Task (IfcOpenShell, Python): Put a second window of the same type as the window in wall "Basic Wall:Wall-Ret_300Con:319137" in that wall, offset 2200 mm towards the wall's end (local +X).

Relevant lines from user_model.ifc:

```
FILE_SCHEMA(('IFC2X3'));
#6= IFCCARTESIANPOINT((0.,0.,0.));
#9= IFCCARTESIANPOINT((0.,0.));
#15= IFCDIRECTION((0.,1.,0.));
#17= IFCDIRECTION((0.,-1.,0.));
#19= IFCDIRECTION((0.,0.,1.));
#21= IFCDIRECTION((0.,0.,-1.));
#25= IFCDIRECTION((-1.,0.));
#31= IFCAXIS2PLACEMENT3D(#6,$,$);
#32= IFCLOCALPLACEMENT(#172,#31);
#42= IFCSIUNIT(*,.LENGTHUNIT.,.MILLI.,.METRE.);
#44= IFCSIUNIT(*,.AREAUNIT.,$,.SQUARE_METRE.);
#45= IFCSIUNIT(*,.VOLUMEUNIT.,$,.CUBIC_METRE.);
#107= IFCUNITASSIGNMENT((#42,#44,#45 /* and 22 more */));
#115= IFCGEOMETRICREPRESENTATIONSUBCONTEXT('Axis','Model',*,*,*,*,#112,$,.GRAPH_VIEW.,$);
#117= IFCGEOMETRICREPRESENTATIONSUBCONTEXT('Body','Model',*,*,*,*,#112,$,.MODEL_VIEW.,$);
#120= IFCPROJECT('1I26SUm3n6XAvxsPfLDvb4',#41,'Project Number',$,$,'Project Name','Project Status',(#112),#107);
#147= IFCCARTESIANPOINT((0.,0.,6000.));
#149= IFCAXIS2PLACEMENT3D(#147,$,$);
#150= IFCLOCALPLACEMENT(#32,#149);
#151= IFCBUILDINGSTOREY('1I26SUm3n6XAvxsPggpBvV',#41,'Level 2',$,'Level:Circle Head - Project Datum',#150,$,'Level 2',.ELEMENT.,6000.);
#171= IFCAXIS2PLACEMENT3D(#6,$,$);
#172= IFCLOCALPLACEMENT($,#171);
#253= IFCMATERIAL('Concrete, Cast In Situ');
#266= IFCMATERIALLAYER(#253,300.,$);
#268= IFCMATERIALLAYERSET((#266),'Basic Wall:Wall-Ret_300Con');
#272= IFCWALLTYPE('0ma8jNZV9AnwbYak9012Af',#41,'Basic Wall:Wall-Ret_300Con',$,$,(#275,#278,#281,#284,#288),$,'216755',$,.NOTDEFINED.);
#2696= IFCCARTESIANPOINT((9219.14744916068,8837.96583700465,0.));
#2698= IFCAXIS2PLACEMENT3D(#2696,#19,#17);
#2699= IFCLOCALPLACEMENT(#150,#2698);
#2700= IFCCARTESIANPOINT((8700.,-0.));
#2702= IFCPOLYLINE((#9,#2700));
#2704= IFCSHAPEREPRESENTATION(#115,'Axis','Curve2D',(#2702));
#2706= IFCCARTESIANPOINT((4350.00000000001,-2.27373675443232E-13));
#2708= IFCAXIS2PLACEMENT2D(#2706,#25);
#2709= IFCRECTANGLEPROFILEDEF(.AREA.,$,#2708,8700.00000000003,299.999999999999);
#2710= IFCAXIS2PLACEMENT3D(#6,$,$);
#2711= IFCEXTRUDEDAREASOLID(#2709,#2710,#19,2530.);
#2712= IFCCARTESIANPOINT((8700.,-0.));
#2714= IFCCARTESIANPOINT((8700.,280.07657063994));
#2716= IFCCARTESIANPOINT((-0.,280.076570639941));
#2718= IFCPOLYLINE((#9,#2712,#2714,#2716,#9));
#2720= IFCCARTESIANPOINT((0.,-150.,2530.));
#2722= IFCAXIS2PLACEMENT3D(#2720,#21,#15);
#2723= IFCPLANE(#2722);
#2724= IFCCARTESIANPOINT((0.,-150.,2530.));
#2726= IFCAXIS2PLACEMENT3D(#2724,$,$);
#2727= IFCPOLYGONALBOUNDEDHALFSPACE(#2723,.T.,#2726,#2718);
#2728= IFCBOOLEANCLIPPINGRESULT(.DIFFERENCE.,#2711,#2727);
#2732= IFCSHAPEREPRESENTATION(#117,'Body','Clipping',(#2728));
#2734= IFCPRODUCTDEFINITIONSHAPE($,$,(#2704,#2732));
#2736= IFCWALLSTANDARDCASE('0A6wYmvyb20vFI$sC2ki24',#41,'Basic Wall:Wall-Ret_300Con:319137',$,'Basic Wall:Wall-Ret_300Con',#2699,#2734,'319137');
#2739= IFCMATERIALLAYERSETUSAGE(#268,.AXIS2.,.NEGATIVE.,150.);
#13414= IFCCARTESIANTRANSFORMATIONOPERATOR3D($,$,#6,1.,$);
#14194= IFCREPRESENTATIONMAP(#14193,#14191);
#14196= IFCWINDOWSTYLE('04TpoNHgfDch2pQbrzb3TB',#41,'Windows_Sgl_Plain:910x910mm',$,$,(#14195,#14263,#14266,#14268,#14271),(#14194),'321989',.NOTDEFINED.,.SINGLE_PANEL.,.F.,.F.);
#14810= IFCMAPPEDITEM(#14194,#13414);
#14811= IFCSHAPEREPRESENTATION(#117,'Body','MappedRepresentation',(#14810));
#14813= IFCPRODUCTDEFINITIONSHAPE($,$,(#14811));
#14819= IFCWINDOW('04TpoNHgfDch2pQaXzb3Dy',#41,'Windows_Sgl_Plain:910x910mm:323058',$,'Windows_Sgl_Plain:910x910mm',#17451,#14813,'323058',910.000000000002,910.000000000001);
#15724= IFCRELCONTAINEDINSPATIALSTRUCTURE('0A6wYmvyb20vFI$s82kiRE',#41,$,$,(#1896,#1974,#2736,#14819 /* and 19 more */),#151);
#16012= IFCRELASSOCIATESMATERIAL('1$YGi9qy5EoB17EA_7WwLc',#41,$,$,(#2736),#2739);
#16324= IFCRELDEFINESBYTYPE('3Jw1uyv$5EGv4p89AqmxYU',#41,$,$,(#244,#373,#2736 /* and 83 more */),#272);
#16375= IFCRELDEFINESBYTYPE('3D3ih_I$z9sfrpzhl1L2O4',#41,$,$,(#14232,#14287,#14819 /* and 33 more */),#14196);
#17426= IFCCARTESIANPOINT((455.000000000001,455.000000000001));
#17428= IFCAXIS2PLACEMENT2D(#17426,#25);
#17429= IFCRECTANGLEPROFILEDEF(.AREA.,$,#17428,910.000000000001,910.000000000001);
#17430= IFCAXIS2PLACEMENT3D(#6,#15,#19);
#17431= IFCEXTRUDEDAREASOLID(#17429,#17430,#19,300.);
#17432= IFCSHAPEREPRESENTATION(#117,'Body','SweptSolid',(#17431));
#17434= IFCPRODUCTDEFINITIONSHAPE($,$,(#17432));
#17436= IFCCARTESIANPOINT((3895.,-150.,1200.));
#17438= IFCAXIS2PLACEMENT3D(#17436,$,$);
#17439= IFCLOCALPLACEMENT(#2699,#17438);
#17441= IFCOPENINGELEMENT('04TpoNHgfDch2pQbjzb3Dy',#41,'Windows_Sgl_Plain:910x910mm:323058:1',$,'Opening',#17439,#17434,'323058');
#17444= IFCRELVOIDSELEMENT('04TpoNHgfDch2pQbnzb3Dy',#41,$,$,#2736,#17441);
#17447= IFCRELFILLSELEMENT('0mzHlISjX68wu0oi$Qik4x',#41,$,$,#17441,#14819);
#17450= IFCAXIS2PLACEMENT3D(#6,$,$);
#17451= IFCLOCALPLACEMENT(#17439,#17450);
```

```python
import ifcopenshell
import ifcopenshell.api.feature
import ifcopenshell.api.geometry
import ifcopenshell.api.root
import ifcopenshell.geom
import ifcopenshell.util.element
import ifcopenshell.util.placement
import ifcopenshell.util.shape
import ifcopenshell.util.unit

model = ifcopenshell.open("user_model.ifc")
unit_scale = ifcopenshell.util.unit.calculate_unit_scale(model)
settings = ifcopenshell.geom.settings()


def volume(element):
    """Net volume in cubic metres, openings subtracted."""
    shape = ifcopenshell.geom.create_shape(settings, element)
    return ifcopenshell.util.shape.get_volume(shape.geometry)


def reuse_history(source, copy):
    """copy_class also copies each property set's owner history, people and application; keep the originals."""
    for rel in copy.IsDefinedBy:
        if rel.is_a("IfcRelDefinesByProperties") and (history := rel.RelatingPropertyDefinition.OwnerHistory):
            rel.RelatingPropertyDefinition.OwnerHistory = source.OwnerHistory
            ifcopenshell.util.element.remove_deep2(model, history)


window = model.by_guid("04TpoNHgfDch2pQaXzb3Dy")
opening = window.FillsVoids[0].RelatingOpeningElement
wall = opening.VoidsElements[0].RelatingBuildingElement
before = volume(wall)
shift = ifcopenshell.util.placement.get_local_placement(wall.ObjectPlacement)[:3, 0] * 2.2 / unit_scale

# copy_class copies the void relationship, type, container and properties, but no geometry.
new_opening = ifcopenshell.api.root.copy_class(model, product=opening)
new_opening.Representation = ifcopenshell.util.element.copy_deep(
    model, opening.Representation, exclude=["IfcGeometricRepresentationContext", "IfcRepresentationMap"]
)
new_opening.Name = "Windows_Sgl_Plain:910x910mm"
new_opening.Tag = None
new_window = ifcopenshell.api.root.copy_class(model, product=window)
new_window.Representation = ifcopenshell.util.element.copy_deep(
    model, window.Representation, exclude=["IfcGeometricRepresentationContext", "IfcRepresentationMap"]
)
new_window.Name = "Windows_Sgl_Plain:910x910mm"
new_window.Tag = None
reuse_history(window, new_window)
fills = ifcopenshell.api.feature.add_filling(model, opening=new_opening, element=new_window)
fills.OwnerHistory = new_window.OwnerHistory  # required in IFC2X3

for old, new in ((opening, new_opening), (window, new_window)):
    matrix = ifcopenshell.util.placement.get_local_placement(old.ObjectPlacement)
    matrix[:3, 3] += shift
    ifcopenshell.api.geometry.edit_object_placement(model, product=new, matrix=matrix, is_si=False)

after = volume(wall)

print(f"wall volume {before:.3f} -> {after:.3f} m3")

model.write("user_model_edited.ifc")
```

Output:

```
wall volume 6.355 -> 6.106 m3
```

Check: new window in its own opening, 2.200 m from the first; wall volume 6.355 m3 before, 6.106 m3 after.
